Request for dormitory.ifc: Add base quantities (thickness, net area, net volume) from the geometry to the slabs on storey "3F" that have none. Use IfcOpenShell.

First a look at what the model holds.

```python
import ifcopenshell
import ifcopenshell.util.element
import ifcopenshell.util.unit

model = ifcopenshell.open("dormitory.ifc")
print(model.schema)
for unit_type in ("LENGTHUNIT", "AREAUNIT", "VOLUMEUNIT"):
    print(unit_type, ifcopenshell.util.unit.calculate_unit_scale(model, unit_type))
storey = next(s for s in model.by_type("IfcBuildingStorey") if s.Name == "3F")
slabs = [e for e in ifcopenshell.util.element.get_decomposition(storey) if e.is_a("IfcSlab")]
for e in sorted(slabs, key=lambda e: e.id()):
    print(e.id(), e.is_a(), e.Name, list(ifcopenshell.util.element.get_psets(e, qtos_only=True)), sep=" | ")
```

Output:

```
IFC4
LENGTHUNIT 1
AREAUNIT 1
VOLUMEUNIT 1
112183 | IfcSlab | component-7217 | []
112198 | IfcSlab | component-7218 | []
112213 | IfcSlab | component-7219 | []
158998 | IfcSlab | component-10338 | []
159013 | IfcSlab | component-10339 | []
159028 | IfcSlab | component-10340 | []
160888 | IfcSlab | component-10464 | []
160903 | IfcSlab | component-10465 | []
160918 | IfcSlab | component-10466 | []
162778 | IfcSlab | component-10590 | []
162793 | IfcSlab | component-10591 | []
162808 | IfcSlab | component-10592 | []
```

```python
import ifcopenshell
import ifcopenshell.api.pset
import ifcopenshell.geom
import ifcopenshell.util.element
import ifcopenshell.util.shape
import ifcopenshell.util.unit

model = ifcopenshell.open("dormitory.ifc")
unit_scale = ifcopenshell.util.unit.calculate_unit_scale(model)
area_scale = ifcopenshell.util.unit.calculate_unit_scale(model, "AREAUNIT")
volume_scale = ifcopenshell.util.unit.calculate_unit_scale(model, "VOLUMEUNIT")
settings = ifcopenshell.geom.settings()

storey = next(s for s in model.by_type("IfcBuildingStorey") if s.Name == "3F")
slabs = [e for e in ifcopenshell.util.element.get_decomposition(storey) if e.is_a("IfcSlab")]

for e in sorted(slabs, key=lambda e: e.id()):
    if ifcopenshell.util.element.get_psets(e, qtos_only=True, should_inherit=False):
        continue
    # Geometry comes back in metres, in the element's own axes.
    shape = ifcopenshell.geom.create_shape(settings, e)
    values = {
        "Width": ifcopenshell.util.shape.get_z(shape.geometry) / unit_scale,
        "NetArea": ifcopenshell.util.shape.get_footprint_area(shape.geometry) / area_scale,
        "NetVolume": ifcopenshell.util.shape.get_volume(shape.geometry) / volume_scale,
    }
    qto = ifcopenshell.api.pset.add_qto(model, product=e, name="Qto_SlabBaseQuantities")
    ifcopenshell.api.pset.edit_qto(model, qto=qto, properties=values)
    print(e.id(), {k: round(v, 3) for k, v in values.items()})

model.write("dormitory_v2.ifc")
```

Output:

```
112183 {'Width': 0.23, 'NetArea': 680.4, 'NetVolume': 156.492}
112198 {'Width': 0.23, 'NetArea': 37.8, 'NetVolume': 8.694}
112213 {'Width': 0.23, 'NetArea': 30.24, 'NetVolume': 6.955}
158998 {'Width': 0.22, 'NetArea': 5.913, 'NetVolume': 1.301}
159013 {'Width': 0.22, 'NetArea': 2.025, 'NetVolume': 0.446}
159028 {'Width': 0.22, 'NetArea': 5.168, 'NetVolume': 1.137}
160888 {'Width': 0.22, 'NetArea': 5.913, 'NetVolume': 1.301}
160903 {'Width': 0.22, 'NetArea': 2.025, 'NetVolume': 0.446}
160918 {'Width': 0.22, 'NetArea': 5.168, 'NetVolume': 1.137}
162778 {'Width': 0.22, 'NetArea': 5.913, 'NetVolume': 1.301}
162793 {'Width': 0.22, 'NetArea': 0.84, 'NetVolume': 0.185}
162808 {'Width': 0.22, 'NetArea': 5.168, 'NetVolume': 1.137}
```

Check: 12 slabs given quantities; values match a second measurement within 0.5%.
